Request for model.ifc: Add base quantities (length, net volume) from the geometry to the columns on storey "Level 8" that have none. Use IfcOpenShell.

First a look at what the model holds.

```python
import ifcopenshell
import ifcopenshell.util.element
import ifcopenshell.util.unit

model = ifcopenshell.open("model.ifc")
print(model.schema)
for unit_type in ("LENGTHUNIT", "AREAUNIT", "VOLUMEUNIT"):
    print(unit_type, ifcopenshell.util.unit.calculate_unit_scale(model, unit_type))
storey = next(s for s in model.by_type("IfcBuildingStorey") if s.Name == "Level 8")
columns = [e for e in ifcopenshell.util.element.get_decomposition(storey) if e.is_a("IfcColumn")]
for e in sorted(columns, key=lambda e: e.id()):
    print(e.id(), e.is_a(), e.Name, list(ifcopenshell.util.element.get_psets(e, qtos_only=True)), sep=" | ")
```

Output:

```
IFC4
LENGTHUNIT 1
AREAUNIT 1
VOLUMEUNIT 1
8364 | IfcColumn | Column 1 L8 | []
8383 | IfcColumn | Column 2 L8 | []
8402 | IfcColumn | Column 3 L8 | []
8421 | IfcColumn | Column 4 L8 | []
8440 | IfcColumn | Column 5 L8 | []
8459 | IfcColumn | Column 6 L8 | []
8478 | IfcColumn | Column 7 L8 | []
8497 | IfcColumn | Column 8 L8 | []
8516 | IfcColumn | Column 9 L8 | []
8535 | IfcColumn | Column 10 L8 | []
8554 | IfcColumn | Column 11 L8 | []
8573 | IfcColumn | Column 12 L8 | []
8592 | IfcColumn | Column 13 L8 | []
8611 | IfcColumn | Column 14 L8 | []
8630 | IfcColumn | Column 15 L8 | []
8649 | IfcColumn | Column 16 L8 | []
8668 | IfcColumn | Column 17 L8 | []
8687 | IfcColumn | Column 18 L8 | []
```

```python
import ifcopenshell
import ifcopenshell.api.pset
import ifcopenshell.geom
import ifcopenshell.util.element
import ifcopenshell.util.shape
import ifcopenshell.util.unit

model = ifcopenshell.open("model.ifc")
unit_scale = ifcopenshell.util.unit.calculate_unit_scale(model)
volume_scale = ifcopenshell.util.unit.calculate_unit_scale(model, "VOLUMEUNIT")
settings = ifcopenshell.geom.settings()

storey = next(s for s in model.by_type("IfcBuildingStorey") if s.Name == "Level 8")
columns = [e for e in ifcopenshell.util.element.get_decomposition(storey) if e.is_a("IfcColumn")]

for e in sorted(columns, key=lambda e: e.id()):
    if ifcopenshell.util.element.get_psets(e, qtos_only=True, should_inherit=False):
        continue
    # Geometry comes back in metres, in the element's own axes.
    shape = ifcopenshell.geom.create_shape(settings, e)
    values = {
        "Length": ifcopenshell.util.shape.get_z(shape.geometry) / unit_scale,
        "NetVolume": ifcopenshell.util.shape.get_volume(shape.geometry) / volume_scale,
    }
    qto = ifcopenshell.api.pset.add_qto(model, product=e, name="Qto_ColumnBaseQuantities")
    ifcopenshell.api.pset.edit_qto(model, qto=qto, properties=values)
    print(e.id(), {k: round(v, 3) for k, v in values.items()})

model.write("model_updated.ifc")
```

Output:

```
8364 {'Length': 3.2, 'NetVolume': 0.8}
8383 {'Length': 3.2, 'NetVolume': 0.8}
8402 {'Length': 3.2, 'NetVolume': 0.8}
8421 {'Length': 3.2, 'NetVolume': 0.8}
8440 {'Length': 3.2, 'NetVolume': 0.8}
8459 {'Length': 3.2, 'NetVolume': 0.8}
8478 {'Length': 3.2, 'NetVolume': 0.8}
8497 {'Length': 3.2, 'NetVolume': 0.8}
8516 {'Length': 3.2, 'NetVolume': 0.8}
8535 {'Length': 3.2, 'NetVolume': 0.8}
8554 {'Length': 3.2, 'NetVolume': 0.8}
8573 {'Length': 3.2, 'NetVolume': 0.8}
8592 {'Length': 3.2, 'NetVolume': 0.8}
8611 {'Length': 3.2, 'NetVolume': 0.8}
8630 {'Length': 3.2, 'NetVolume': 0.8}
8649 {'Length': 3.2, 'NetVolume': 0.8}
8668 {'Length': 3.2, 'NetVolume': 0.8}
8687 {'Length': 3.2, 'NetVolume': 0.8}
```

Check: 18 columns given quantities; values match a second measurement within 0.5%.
